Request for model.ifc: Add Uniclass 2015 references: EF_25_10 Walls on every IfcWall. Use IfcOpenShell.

First a look at what the model holds.

```python
import ifcopenshell

model = ifcopenshell.open("model.ifc")
print(model.schema)
print("classifications:", [c.Name for c in model.by_type("IfcClassification")])
for ifc_class in ("IfcDoor", "IfcRoof", "IfcStair", "IfcWall", "IfcWindow"):
    print(ifc_class, len(model.by_type(ifc_class)))
```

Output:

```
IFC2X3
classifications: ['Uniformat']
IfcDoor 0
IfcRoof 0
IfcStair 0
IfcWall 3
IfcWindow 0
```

```python
import ifcopenshell
import ifcopenshell.api.classification

model = ifcopenshell.open("model.ifc")

# IFC2X3 requires Source and Edition and has no link from the project to the system.
system = model.create_entity("IfcClassification", Source="NBS", Edition="2015", Name="Uniclass 2015")

codes = {
    "IfcWall": ("EF_25_10", "Walls"),
}
for ifc_class, (code, name) in codes.items():
    products = model.by_type(ifc_class)
    ifcopenshell.api.classification.add_reference(
        model, products=products, classification=system, identification=code, name=name
    )
    print(code, len(products))

model.write("model_rev.ifc")
```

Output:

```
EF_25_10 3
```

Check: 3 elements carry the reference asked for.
